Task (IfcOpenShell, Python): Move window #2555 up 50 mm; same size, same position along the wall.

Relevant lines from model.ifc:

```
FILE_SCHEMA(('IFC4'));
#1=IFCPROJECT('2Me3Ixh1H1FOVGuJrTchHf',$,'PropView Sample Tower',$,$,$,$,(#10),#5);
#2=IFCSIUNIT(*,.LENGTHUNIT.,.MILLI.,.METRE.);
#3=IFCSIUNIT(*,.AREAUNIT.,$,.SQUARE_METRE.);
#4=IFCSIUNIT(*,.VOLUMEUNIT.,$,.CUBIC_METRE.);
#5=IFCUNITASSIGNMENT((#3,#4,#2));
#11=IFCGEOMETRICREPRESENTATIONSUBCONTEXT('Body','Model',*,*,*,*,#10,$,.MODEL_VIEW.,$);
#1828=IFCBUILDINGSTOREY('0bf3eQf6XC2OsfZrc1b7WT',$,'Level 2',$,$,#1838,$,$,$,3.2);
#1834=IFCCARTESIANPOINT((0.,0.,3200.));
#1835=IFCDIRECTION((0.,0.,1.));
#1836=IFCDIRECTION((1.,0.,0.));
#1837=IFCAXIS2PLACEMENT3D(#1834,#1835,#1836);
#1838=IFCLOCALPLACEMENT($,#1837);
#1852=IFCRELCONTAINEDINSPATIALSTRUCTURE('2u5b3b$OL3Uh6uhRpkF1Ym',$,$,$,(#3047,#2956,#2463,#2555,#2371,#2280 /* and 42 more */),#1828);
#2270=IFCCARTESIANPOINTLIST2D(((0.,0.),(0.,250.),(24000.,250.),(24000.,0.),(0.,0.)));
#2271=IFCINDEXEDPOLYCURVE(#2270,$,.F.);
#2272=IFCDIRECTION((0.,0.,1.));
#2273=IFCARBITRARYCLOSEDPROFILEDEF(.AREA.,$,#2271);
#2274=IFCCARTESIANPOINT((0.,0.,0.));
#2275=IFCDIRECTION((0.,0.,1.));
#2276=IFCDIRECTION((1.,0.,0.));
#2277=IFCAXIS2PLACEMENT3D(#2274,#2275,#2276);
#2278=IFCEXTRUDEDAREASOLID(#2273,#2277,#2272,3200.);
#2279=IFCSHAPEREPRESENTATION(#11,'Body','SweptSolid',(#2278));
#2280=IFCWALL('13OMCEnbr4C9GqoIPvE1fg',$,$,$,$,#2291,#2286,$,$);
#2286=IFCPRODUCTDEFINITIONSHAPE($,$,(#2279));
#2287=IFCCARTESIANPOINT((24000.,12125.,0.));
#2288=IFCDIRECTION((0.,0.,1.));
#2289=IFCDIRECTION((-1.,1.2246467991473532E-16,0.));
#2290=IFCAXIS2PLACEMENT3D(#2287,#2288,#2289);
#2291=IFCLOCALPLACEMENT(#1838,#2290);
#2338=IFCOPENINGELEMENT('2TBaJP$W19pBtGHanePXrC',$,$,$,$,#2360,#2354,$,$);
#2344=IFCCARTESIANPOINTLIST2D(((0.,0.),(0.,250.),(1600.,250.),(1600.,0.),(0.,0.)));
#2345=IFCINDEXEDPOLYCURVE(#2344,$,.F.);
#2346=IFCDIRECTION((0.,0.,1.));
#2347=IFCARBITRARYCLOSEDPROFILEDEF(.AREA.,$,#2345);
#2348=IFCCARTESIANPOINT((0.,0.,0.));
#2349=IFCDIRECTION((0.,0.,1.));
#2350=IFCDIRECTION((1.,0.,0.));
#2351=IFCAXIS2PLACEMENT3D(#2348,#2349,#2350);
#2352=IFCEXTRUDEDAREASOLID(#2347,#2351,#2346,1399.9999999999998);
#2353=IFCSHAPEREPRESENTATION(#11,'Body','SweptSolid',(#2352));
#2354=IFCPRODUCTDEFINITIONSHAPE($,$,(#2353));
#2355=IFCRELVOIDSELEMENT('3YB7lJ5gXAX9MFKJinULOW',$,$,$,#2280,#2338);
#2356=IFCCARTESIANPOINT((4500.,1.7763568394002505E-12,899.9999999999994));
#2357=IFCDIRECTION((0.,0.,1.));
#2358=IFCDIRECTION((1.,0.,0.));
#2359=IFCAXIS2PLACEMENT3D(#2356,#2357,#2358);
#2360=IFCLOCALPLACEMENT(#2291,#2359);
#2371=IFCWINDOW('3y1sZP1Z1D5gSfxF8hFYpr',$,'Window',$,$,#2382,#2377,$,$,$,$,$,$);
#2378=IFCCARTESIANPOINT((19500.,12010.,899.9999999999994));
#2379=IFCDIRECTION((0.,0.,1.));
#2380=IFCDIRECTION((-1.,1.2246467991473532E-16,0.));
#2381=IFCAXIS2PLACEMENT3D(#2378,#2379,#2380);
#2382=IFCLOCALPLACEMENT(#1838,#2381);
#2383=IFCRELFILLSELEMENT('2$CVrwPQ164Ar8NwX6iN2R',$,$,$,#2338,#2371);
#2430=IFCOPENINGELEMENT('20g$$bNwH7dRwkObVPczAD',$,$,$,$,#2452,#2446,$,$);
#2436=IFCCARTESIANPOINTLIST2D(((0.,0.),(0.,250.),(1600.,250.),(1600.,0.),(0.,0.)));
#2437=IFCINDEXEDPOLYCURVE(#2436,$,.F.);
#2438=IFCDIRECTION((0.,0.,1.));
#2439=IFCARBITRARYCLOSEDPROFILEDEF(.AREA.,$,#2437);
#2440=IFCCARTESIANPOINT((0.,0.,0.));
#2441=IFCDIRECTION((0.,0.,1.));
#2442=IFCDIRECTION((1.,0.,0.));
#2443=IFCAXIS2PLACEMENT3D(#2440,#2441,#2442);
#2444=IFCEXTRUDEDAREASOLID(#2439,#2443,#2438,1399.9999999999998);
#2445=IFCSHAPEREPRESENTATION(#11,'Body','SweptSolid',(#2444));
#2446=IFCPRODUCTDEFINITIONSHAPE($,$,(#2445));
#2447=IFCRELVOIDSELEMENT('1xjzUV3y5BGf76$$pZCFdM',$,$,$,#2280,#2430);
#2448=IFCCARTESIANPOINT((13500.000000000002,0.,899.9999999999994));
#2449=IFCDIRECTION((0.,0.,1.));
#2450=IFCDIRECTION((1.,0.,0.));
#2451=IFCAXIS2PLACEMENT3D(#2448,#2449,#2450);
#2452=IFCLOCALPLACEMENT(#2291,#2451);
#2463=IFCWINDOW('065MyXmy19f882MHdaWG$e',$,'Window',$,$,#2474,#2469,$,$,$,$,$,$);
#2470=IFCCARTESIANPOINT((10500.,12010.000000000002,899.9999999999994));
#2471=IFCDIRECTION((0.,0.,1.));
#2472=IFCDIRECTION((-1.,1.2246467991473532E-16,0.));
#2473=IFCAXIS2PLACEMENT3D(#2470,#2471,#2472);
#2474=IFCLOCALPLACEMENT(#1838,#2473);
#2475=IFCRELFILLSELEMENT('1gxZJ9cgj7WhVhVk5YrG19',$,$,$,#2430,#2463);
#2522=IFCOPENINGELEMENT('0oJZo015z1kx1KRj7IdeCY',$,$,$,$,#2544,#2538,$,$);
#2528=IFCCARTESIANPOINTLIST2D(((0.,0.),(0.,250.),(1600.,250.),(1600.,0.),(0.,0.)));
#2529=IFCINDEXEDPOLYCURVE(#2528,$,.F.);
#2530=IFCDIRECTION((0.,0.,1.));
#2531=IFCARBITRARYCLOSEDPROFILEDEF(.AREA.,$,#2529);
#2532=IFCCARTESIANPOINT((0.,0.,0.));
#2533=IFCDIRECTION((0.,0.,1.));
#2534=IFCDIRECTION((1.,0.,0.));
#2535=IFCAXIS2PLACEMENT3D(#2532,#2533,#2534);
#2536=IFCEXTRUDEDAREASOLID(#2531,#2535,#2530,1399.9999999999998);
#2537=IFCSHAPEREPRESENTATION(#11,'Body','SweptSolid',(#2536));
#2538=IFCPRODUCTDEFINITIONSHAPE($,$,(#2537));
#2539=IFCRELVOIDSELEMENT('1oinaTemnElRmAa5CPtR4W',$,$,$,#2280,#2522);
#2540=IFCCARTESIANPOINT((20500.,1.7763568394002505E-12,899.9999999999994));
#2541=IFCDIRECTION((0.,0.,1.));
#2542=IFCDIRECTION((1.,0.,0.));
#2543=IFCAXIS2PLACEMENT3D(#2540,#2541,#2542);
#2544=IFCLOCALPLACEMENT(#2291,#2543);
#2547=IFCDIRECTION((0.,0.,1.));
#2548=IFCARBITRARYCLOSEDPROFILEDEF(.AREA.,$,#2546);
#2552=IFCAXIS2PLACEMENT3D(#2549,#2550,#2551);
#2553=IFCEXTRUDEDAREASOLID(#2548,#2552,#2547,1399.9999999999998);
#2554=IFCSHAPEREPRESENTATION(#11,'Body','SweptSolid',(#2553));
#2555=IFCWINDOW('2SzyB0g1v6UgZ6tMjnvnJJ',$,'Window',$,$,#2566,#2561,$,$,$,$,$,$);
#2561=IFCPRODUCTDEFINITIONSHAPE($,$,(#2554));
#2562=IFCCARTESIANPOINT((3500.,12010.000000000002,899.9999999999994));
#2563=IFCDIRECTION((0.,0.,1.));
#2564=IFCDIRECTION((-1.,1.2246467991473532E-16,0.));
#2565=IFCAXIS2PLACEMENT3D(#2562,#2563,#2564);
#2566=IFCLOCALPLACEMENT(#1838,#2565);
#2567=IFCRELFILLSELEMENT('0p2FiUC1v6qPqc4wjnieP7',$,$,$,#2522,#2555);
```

```python
import numpy as np
import ifcopenshell
import ifcopenshell.api.geometry
import ifcopenshell.util.placement
import ifcopenshell.util.unit

model = ifcopenshell.open("model.ifc")
unit_scale = ifcopenshell.util.unit.calculate_unit_scale(model)

window = model.by_id(2555)
opening = window.FillsVoids[0].RelatingOpeningElement
dz = 0.05 / unit_scale

shift = np.array([0.0, 0.0, dz])
# The window is not placed relative to its opening, so move both.
for product in (opening, window):
    matrix = ifcopenshell.util.placement.get_local_placement(product.ObjectPlacement)
    matrix[:3, 3] += shift
    ifcopenshell.api.geometry.edit_object_placement(model, product=product, matrix=matrix, is_si=False)

print(f"moved by {dz * unit_scale:+.3f} m")

model.write("model_updated.ifc")
```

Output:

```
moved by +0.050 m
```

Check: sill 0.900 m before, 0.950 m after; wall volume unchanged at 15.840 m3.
